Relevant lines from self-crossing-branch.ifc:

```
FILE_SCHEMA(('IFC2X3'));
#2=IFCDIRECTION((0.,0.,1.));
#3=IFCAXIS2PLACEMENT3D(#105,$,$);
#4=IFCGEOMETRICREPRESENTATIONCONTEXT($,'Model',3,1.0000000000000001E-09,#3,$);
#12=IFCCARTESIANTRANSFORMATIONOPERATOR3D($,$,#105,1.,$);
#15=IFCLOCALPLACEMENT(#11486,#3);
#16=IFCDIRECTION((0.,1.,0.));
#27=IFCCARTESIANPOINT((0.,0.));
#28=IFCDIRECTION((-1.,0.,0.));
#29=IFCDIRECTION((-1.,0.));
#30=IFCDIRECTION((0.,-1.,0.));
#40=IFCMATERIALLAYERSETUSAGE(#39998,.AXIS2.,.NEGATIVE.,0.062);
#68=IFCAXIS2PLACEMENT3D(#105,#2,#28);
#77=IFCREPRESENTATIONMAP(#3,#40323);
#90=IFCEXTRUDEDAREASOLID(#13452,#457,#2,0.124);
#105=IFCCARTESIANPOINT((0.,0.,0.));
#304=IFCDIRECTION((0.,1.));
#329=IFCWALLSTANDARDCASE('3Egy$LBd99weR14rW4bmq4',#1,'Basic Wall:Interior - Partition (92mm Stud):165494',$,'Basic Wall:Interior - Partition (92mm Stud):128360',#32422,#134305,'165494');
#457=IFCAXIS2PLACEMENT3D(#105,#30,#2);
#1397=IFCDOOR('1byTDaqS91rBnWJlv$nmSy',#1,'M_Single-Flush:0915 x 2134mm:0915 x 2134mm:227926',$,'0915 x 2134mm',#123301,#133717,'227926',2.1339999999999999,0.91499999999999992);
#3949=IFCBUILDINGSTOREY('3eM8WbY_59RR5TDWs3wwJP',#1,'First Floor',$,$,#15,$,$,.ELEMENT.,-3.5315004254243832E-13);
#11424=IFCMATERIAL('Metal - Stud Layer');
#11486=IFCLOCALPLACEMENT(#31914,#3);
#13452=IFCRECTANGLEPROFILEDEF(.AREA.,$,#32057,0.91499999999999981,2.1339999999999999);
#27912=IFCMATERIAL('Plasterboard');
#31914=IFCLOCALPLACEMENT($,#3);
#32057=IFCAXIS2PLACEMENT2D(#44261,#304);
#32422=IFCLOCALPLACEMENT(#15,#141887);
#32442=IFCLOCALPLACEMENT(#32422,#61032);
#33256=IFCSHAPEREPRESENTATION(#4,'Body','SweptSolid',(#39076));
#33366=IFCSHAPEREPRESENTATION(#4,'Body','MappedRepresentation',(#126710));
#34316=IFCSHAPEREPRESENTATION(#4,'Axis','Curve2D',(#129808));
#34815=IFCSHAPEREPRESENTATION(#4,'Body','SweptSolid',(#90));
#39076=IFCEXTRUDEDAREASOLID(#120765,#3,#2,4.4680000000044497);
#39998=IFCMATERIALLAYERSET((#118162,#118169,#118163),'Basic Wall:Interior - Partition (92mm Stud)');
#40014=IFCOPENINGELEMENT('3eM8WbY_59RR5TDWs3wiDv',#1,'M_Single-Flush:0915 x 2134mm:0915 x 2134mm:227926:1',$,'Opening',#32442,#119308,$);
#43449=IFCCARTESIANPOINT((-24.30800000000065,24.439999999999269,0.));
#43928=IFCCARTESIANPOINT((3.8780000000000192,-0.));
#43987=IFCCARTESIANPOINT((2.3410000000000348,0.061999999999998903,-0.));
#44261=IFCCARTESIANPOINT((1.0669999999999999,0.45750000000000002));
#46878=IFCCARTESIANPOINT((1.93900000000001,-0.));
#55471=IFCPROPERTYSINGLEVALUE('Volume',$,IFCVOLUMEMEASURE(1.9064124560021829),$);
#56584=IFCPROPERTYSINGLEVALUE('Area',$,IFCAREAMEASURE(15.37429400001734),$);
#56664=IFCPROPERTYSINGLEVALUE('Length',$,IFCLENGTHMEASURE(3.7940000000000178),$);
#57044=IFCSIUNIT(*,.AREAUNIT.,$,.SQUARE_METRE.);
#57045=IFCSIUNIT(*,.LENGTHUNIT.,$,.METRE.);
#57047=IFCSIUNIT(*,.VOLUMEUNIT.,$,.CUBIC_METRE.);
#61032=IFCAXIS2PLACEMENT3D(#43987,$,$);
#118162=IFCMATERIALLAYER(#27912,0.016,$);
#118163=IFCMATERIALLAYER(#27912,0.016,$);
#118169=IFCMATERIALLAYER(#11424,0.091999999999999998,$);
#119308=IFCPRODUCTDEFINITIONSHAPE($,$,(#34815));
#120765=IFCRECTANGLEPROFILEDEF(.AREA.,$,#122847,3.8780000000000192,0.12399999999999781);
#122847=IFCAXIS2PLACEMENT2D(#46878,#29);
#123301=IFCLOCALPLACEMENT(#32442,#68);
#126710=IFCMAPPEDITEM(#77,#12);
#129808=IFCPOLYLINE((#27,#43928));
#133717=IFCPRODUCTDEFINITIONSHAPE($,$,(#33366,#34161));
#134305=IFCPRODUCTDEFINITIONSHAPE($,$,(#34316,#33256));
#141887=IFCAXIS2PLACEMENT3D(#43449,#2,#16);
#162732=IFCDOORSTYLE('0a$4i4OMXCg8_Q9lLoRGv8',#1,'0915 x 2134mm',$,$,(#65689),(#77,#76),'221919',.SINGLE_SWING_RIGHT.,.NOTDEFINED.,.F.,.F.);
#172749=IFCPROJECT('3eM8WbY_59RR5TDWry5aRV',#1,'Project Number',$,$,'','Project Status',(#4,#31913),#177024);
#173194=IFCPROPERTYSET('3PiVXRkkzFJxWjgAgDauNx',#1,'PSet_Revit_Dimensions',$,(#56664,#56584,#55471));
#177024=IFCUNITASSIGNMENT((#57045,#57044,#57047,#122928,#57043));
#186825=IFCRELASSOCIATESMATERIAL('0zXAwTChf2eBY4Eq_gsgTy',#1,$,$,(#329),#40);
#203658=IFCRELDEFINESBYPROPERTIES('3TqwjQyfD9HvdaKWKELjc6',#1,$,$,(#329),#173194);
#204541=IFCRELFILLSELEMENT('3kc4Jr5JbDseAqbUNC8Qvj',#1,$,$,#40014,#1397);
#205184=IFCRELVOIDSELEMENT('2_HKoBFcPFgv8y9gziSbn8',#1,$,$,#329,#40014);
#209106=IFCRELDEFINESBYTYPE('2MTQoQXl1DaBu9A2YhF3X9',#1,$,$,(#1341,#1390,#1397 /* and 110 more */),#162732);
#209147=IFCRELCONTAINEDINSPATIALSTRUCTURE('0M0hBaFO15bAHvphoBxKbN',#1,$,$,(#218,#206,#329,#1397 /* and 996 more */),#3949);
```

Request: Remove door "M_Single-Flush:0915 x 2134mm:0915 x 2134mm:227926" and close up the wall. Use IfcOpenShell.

```python
import ifcopenshell
import ifcopenshell.api.feature
import ifcopenshell.api.pset
import ifcopenshell.api.root
import ifcopenshell.geom
import ifcopenshell.util.element
import ifcopenshell.util.shape
import ifcopenshell.util.unit

model = ifcopenshell.open("self-crossing-branch.ifc")
area_scale = ifcopenshell.util.unit.calculate_unit_scale(model, "AREAUNIT")
volume_scale = ifcopenshell.util.unit.calculate_unit_scale(model, "VOLUMEUNIT")
settings = ifcopenshell.geom.settings()


def volume(element):
    """Net volume in cubic metres, openings subtracted."""
    shape = ifcopenshell.geom.create_shape(settings, element)
    return ifcopenshell.util.shape.get_volume(shape.geometry)


door = model.by_guid("1byTDaqS91rBnWJlv$nmSy")
opening = door.FillsVoids[0].RelatingOpeningElement
wall = opening.VoidsElements[0].RelatingBuildingElement
before = volume(wall)

ifcopenshell.api.root.remove_product(model, product=door)
ifcopenshell.api.feature.remove_feature(model, feature=opening)

after = volume(wall)
thickness = 0.124  # wall thickness in metres

# Update the wall's stored quantities.
pset = model.by_id(ifcopenshell.util.element.get_pset(wall, "PSet_Revit_Dimensions", should_inherit=False)["id"])
ifcopenshell.api.pset.edit_pset(model, pset=pset, properties={
    "Area": model.create_entity("IfcAreaMeasure", after / thickness / area_scale),
    "Volume": model.create_entity("IfcVolumeMeasure", after / volume_scale),
})

print(f"wall volume {before:.3f} -> {after:.3f} m3")

model.write("self-crossing-branch_updated.ifc")
```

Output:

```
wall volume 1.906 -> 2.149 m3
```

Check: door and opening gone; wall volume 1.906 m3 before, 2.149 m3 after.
